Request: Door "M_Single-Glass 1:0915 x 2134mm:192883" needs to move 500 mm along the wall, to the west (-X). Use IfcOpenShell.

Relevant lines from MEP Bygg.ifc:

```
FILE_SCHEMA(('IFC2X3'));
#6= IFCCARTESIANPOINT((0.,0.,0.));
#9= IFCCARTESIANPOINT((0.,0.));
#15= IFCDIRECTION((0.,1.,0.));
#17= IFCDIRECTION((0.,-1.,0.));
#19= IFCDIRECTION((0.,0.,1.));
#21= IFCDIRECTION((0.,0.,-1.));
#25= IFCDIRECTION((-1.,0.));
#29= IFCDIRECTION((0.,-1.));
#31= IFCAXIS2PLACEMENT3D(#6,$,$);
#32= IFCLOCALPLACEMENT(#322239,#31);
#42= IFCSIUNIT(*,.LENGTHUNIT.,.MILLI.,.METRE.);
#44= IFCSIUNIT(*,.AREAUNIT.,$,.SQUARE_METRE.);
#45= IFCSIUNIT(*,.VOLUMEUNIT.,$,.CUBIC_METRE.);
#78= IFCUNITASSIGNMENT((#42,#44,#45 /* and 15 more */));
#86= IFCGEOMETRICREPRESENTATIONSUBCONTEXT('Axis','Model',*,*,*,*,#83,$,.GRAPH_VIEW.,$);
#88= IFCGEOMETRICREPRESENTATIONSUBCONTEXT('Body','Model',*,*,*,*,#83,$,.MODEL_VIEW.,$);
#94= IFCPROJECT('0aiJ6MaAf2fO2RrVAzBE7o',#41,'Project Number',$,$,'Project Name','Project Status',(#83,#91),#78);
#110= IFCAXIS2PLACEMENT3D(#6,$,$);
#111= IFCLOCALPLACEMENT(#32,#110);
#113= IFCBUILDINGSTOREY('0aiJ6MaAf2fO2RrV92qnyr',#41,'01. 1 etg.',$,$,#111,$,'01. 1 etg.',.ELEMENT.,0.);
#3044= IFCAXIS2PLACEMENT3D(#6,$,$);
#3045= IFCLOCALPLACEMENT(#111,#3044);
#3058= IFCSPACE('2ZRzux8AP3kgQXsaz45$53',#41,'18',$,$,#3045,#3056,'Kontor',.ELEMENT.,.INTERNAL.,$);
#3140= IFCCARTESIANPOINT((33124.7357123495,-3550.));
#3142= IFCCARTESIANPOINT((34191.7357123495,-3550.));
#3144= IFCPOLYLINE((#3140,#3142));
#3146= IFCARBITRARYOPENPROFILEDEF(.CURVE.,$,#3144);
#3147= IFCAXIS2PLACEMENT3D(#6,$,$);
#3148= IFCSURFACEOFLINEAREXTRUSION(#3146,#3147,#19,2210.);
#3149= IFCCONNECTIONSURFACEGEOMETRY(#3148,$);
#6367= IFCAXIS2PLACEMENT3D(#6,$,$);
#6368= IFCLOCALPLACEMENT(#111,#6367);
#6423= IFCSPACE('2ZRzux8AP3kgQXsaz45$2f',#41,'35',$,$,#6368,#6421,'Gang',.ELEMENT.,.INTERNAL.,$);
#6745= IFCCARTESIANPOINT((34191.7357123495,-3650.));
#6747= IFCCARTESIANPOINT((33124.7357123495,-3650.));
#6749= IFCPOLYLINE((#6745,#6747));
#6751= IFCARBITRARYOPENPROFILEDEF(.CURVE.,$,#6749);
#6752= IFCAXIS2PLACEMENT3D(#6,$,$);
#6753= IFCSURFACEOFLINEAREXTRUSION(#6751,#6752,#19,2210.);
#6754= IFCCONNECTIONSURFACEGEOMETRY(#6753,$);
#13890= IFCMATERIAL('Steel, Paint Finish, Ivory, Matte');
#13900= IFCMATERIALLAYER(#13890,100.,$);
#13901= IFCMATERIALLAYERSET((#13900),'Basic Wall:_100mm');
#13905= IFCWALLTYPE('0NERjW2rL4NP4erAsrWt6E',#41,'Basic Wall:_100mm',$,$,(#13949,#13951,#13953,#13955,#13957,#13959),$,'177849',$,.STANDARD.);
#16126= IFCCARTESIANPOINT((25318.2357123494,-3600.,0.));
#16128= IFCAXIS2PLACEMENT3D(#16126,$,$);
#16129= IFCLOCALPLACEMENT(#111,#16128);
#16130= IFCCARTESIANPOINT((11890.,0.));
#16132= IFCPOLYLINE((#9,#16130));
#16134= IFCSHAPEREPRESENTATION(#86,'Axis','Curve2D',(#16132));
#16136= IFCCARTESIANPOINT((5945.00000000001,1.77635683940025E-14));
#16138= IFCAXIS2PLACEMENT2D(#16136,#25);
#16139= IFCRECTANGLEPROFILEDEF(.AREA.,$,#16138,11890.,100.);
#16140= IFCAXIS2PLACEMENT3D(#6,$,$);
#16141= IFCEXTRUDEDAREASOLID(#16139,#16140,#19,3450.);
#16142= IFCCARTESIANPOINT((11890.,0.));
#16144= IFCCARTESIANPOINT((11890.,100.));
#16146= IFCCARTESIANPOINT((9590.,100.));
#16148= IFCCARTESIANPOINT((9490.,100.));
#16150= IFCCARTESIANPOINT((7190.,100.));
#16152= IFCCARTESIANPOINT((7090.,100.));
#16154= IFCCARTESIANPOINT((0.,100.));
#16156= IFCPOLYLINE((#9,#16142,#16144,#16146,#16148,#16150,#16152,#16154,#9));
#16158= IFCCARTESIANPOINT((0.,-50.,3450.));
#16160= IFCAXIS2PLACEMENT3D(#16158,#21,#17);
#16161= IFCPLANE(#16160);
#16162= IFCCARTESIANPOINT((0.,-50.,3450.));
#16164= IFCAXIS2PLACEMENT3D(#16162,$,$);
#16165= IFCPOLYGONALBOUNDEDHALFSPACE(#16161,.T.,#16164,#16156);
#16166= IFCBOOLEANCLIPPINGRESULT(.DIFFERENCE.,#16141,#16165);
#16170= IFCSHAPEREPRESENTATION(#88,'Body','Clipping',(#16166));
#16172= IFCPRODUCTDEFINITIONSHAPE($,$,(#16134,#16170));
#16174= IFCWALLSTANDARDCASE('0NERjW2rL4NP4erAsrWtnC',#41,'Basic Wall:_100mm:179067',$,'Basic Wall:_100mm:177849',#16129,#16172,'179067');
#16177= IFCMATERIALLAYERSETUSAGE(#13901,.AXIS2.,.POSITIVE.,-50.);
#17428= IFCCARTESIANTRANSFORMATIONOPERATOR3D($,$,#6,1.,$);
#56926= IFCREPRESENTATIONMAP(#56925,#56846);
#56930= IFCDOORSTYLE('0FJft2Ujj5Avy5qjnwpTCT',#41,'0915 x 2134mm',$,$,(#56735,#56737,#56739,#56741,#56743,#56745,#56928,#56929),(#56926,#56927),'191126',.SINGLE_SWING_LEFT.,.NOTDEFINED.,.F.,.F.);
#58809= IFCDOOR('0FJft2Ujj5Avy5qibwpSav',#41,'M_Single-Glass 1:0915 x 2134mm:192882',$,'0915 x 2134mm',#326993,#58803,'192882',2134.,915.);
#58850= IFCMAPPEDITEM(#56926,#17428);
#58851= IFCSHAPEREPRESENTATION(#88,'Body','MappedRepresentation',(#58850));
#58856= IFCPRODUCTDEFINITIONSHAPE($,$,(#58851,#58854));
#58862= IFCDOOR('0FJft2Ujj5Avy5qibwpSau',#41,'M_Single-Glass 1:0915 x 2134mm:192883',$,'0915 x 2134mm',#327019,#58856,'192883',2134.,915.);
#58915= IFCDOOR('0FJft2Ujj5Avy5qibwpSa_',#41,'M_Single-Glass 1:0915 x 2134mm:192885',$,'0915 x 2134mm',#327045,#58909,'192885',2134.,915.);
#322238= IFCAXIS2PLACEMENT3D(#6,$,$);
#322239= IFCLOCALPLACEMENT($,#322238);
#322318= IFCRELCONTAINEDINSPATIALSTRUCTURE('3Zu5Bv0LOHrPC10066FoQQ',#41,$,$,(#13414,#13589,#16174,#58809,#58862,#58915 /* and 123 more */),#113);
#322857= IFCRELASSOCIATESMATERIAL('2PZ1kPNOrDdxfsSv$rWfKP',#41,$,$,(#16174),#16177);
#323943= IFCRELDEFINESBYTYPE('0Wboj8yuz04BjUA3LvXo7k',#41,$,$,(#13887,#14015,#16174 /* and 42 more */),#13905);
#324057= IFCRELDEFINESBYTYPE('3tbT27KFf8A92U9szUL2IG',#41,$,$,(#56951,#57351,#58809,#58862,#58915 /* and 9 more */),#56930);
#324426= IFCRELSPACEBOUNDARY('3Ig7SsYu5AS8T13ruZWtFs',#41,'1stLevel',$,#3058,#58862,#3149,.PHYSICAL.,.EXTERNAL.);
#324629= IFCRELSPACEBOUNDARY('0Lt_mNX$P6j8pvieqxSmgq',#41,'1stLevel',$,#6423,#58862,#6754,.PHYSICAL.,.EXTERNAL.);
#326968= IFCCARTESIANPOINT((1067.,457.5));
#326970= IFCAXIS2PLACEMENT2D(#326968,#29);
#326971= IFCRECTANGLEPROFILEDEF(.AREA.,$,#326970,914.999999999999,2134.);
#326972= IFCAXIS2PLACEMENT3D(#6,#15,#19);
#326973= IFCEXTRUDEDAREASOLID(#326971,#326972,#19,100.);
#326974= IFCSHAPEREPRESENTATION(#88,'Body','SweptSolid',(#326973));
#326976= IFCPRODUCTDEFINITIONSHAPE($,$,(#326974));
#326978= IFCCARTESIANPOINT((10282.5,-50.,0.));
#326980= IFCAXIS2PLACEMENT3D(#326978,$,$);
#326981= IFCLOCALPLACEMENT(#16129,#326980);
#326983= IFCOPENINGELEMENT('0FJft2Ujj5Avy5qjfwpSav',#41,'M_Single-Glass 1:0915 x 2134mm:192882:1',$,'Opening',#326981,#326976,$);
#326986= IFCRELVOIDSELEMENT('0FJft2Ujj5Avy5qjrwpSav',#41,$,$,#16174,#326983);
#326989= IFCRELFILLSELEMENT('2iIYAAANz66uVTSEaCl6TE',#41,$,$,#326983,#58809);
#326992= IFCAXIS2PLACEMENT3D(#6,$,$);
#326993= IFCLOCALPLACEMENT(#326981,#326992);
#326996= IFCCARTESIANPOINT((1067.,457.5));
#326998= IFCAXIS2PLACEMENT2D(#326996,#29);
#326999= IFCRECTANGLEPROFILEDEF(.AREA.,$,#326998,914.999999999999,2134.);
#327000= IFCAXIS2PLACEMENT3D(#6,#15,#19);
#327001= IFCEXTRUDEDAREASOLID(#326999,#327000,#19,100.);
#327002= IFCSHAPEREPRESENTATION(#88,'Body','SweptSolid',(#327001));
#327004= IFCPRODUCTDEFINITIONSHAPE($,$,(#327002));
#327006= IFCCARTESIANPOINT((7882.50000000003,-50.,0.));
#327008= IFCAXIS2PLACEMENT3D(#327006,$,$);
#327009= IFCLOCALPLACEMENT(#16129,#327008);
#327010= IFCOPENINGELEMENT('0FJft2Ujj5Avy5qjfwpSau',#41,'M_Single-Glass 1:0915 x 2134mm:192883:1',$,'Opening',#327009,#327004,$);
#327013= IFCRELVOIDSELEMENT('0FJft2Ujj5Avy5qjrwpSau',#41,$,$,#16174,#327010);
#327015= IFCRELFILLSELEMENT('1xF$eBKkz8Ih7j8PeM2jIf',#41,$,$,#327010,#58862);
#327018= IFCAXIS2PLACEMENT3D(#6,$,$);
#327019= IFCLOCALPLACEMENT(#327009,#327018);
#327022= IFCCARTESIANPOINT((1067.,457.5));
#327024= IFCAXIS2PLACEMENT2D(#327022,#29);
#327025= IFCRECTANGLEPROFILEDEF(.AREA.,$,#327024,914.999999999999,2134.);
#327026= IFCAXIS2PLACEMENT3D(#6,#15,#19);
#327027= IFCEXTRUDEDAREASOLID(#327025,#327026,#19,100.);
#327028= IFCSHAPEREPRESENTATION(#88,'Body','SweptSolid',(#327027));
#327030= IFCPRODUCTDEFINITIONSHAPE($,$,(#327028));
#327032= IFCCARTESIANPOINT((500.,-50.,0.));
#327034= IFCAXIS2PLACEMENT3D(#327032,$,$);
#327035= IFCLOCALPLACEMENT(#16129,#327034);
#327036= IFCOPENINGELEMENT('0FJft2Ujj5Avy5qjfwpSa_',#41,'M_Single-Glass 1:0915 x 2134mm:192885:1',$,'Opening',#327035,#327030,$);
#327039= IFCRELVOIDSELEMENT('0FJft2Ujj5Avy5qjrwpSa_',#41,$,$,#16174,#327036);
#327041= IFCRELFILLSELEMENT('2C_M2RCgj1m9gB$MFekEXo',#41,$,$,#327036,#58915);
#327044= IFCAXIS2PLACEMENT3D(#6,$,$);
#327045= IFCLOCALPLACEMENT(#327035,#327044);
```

```python
import numpy as np
import ifcopenshell
import ifcopenshell.api.geometry
import ifcopenshell.util.placement
import ifcopenshell.util.unit

model = ifcopenshell.open("MEP Bygg.ifc")
unit_scale = ifcopenshell.util.unit.calculate_unit_scale(model)

door = model.by_guid("0FJft2Ujj5Avy5qibwpSau")
opening = door.FillsVoids[0].RelatingOpeningElement
wall = opening.VoidsElements[0].RelatingBuildingElement

wall_matrix = ifcopenshell.util.placement.get_local_placement(wall.ObjectPlacement)
shift = wall_matrix[:3, 0] * -0.5 / unit_scale
before = ifcopenshell.util.placement.get_local_placement(door.ObjectPlacement)[:3, 3].copy()

# The door is placed relative to its opening, so it follows when the opening moves.
matrix = ifcopenshell.util.placement.get_local_placement(opening.ObjectPlacement)
matrix[:3, 3] += shift
ifcopenshell.api.geometry.edit_object_placement(
    model, product=opening, matrix=matrix, is_si=False, should_transform_children=True
)

# Space boundary surfaces are stored in each space's coordinates; move them too.
for rel in door.ProvidesBoundaries:
    if not rel.ConnectionGeometry:
        continue
    surface = rel.ConnectionGeometry.SurfaceOnRelatingElement
    space_matrix = ifcopenshell.util.placement.get_local_placement(rel.RelatingSpace.ObjectPlacement)
    point = np.array(surface.Position.Location.Coordinates) + space_matrix[:3, :3].T @ shift
    surface.Position = model.createIfcAxis2Placement3D(
        model.createIfcCartesianPoint(point.tolist()), surface.Position.Axis, surface.Position.RefDirection
    )

after = ifcopenshell.util.placement.get_local_placement(door.ObjectPlacement)[:3, 3]
print("door moved by", (after - before).round(3) + 0.0)

model.write("MEP Bygg_edited.ifc")
```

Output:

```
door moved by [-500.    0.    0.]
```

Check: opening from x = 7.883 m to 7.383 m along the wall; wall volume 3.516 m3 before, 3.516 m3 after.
